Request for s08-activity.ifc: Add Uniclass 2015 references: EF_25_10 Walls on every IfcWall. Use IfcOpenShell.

First a look at what the model holds.

```python
import ifcopenshell

model = ifcopenshell.open("s08-activity.ifc")
print(model.schema)
print("classifications:", [c.Name for c in model.by_type("IfcClassification")])
for ifc_class in ("IfcDoor", "IfcRoof", "IfcStair", "IfcWall", "IfcWindow"):
    print(ifc_class, len(model.by_type(ifc_class)))
```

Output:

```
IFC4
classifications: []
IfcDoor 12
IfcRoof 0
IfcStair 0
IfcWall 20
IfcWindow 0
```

```python
import ifcopenshell
import ifcopenshell.api.classification

model = ifcopenshell.open("s08-activity.ifc")

system = ifcopenshell.api.classification.add_classification(model, classification="Uniclass 2015")

codes = {
    "IfcWall": ("EF_25_10", "Walls"),
}
for ifc_class, (code, name) in codes.items():
    products = model.by_type(ifc_class)
    ifcopenshell.api.classification.add_reference(
        model, products=products, classification=system, identification=code, name=name
    )
    print(code, len(products))

model.write("s08-activity-out.ifc")
```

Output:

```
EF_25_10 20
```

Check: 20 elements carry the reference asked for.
